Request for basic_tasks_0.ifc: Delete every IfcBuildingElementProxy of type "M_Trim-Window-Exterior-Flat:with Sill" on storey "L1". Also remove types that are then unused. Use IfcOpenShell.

First a look at what the model holds.

```python
import ifcopenshell
import ifcopenshell.util.element

model = ifcopenshell.open("basic_tasks_0.ifc")
print(model.schema)
storey = next(s for s in model.by_type("IfcBuildingStorey") if s.Name == "L1")
proxies = [e for e in ifcopenshell.util.element.get_decomposition(storey) if e.is_a("IfcBuildingElementProxy")]
seen = {}
for e in proxies:
    element_type = ifcopenshell.util.element.get_type(e)
    name = element_type.Name if element_type not in (None, e) else None
    seen[name] = seen.get(name, 0) + 1
for name, count in sorted(seen.items(), key=str):
    print(count, "x", name)
```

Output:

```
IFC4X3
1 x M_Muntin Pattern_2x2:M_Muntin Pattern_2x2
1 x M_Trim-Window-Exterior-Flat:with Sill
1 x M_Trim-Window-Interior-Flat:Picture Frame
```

```python
import ifcopenshell
import ifcopenshell.api.root
import ifcopenshell.util.element

model = ifcopenshell.open("basic_tasks_0.ifc")

storey = next(s for s in model.by_type("IfcBuildingStorey") if s.Name == "L1")
proxies = [e for e in ifcopenshell.util.element.get_decomposition(storey) if e.is_a("IfcBuildingElementProxy")]
targets = [e for e in proxies if (t := ifcopenshell.util.element.get_type(e)) not in (None, e) and t.Name == "M_Trim-Window-Exterior-Flat:with Sill"]
types = {ifcopenshell.util.element.get_type(e) for e in targets} - {None, *targets}

for e in targets:
    ifcopenshell.api.root.remove_product(model, product=e)
print(len(targets), "removed")

unused = [t for t in types if not ifcopenshell.util.element.get_types(t)]
for t in unused:
    ifcopenshell.api.root.remove_product(model, product=t)
print(len(unused), "unused types removed")

model.write("basic_tasks_0_updated.ifc")
```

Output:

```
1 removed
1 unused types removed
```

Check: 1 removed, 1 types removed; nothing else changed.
